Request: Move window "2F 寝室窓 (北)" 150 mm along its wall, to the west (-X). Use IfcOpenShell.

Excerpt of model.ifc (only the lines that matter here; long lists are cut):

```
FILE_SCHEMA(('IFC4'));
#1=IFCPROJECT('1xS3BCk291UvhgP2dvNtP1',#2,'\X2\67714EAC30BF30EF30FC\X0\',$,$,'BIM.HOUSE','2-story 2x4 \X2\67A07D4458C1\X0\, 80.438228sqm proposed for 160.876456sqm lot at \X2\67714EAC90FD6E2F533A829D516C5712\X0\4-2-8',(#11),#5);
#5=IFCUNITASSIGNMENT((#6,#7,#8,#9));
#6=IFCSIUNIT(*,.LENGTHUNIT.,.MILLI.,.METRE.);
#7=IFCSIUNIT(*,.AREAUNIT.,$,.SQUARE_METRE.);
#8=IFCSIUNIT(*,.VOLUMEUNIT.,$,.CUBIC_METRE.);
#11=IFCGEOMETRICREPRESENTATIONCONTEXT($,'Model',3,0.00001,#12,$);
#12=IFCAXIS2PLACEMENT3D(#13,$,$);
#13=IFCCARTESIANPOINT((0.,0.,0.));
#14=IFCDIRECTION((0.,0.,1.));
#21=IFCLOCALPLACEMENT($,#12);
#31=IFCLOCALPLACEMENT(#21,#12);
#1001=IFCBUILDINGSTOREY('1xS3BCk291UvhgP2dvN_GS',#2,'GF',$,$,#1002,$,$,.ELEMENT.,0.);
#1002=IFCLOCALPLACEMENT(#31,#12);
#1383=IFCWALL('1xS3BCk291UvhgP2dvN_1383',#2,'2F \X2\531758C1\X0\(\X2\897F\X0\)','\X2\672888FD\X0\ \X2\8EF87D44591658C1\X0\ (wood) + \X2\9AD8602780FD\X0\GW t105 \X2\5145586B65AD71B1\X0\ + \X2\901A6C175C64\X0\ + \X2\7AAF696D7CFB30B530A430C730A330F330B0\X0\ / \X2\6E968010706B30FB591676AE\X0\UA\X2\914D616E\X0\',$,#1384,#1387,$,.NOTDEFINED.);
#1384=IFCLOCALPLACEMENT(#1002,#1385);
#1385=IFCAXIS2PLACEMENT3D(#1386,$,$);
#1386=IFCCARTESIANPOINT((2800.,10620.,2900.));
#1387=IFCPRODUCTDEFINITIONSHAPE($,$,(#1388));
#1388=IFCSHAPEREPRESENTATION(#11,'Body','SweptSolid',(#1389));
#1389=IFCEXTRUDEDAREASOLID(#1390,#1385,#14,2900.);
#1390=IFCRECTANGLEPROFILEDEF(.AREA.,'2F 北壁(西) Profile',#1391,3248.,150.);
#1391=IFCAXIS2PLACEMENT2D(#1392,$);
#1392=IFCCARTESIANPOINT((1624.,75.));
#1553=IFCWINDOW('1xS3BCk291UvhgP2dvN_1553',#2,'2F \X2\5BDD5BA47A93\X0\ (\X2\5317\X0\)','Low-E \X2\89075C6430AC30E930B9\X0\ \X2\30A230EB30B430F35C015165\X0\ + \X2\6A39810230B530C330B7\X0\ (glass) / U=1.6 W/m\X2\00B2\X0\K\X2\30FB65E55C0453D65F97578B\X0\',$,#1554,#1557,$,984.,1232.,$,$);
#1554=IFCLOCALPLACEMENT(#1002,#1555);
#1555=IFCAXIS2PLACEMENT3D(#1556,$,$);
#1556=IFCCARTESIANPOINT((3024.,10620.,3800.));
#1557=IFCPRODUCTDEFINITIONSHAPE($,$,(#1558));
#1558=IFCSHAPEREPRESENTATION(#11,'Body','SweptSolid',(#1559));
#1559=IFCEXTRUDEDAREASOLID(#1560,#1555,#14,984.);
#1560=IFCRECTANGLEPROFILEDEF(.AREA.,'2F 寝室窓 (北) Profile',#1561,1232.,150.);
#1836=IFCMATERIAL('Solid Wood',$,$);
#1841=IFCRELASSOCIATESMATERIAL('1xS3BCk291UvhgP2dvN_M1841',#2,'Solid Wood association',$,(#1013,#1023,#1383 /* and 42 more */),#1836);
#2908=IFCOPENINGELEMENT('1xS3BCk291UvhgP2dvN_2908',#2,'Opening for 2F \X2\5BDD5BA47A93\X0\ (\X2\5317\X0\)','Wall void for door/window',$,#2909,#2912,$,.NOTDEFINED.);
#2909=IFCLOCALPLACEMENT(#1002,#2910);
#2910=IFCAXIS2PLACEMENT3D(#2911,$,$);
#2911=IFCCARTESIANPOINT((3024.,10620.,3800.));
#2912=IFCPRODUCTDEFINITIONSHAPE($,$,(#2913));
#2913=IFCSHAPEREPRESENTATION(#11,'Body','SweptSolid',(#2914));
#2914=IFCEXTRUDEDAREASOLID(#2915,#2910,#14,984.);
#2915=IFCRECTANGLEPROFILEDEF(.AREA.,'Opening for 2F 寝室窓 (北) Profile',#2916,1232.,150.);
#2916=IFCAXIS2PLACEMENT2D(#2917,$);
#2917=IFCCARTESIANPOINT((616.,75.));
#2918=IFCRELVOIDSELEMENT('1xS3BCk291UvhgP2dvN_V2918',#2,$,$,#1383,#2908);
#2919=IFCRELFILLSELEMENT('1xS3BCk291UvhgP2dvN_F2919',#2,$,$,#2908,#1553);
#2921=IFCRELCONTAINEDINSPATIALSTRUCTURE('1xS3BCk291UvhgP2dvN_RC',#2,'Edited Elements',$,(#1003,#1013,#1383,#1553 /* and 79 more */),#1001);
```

```python
import ifcopenshell
import ifcopenshell.api.geometry
import ifcopenshell.util.placement
import ifcopenshell.util.unit

model = ifcopenshell.open("model.ifc")
unit_scale = ifcopenshell.util.unit.calculate_unit_scale(model)

window = model.by_id(1553)
opening = window.FillsVoids[0].RelatingOpeningElement
wall = opening.VoidsElements[0].RelatingBuildingElement

wall_matrix = ifcopenshell.util.placement.get_local_placement(wall.ObjectPlacement)
shift = wall_matrix[:3, 0] * -0.15 / unit_scale
before = ifcopenshell.util.placement.get_local_placement(window.ObjectPlacement)[:3, 3].copy()

# The window is not placed relative to its opening, so move both.
for product in (opening, window):
    matrix = ifcopenshell.util.placement.get_local_placement(product.ObjectPlacement)
    matrix[:3, 3] += shift
    ifcopenshell.api.geometry.edit_object_placement(model, product=product, matrix=matrix, is_si=False)

after = ifcopenshell.util.placement.get_local_placement(window.ObjectPlacement)[:3, 3]
print("window moved by", (after - before).round(3) + 0.0)

model.write("model_v2.ifc")
```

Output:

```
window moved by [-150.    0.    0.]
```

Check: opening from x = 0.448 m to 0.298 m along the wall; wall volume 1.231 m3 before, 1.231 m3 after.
